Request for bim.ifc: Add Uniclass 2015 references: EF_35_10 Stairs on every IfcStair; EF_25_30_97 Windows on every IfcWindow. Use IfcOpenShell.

First a look at what the model holds.

```python
import ifcopenshell

model = ifcopenshell.open("bim.ifc")
print(model.schema)
print("classifications:", [c.Name for c in model.by_type("IfcClassification")])
for ifc_class in ("IfcDoor", "IfcRoof", "IfcStair", "IfcWall", "IfcWindow"):
    print(ifc_class, len(model.by_type(ifc_class)))
```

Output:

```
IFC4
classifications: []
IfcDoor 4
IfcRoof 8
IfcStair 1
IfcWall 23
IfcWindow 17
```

```python
import ifcopenshell
import ifcopenshell.api.classification

model = ifcopenshell.open("bim.ifc")

system = ifcopenshell.api.classification.add_classification(model, classification="Uniclass 2015")

codes = {
    "IfcStair": ("EF_35_10", "Stairs"),
    "IfcWindow": ("EF_25_30_97", "Windows"),
}
for ifc_class, (code, name) in codes.items():
    products = model.by_type(ifc_class)
    ifcopenshell.api.classification.add_reference(
        model, products=products, classification=system, identification=code, name=name
    )
    print(code, len(products))

model.write("bim_updated.ifc")
```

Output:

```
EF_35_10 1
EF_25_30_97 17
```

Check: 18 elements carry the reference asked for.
